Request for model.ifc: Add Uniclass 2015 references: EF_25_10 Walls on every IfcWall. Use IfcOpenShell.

First a look at what the model holds.

```python
import ifcopenshell

model = ifcopenshell.open("model.ifc")
print(model.schema)
print("classifications:", [c.Name for c in model.by_type("IfcClassification")])
for ifc_class in ("IfcDoor", "IfcRoof", "IfcStair", "IfcWall", "IfcWindow"):
    print(ifc_class, len(model.by_type(ifc_class)))
```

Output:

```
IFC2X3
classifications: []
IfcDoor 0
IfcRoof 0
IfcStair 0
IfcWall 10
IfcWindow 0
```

```python
import ifcopenshell
import ifcopenshell.api.classification

model = ifcopenshell.open("model.ifc")

# IFC2X3 requires Source and Edition and has no link from the project to the system.
system = model.create_entity("IfcClassification", Source="NBS", Edition="2015", Name="Uniclass 2015")

codes = {
    "IfcWall": ("EF_25_10", "Walls"),
}
for ifc_class, (code, name) in codes.items():
    products = model.by_type(ifc_class)
    ifcopenshell.api.classification.add_reference(
        model, products=products, classification=system, identification=code, name=name
    )
    print(code, len(products))

model.write("model_updated.ifc")
```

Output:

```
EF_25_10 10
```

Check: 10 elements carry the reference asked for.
